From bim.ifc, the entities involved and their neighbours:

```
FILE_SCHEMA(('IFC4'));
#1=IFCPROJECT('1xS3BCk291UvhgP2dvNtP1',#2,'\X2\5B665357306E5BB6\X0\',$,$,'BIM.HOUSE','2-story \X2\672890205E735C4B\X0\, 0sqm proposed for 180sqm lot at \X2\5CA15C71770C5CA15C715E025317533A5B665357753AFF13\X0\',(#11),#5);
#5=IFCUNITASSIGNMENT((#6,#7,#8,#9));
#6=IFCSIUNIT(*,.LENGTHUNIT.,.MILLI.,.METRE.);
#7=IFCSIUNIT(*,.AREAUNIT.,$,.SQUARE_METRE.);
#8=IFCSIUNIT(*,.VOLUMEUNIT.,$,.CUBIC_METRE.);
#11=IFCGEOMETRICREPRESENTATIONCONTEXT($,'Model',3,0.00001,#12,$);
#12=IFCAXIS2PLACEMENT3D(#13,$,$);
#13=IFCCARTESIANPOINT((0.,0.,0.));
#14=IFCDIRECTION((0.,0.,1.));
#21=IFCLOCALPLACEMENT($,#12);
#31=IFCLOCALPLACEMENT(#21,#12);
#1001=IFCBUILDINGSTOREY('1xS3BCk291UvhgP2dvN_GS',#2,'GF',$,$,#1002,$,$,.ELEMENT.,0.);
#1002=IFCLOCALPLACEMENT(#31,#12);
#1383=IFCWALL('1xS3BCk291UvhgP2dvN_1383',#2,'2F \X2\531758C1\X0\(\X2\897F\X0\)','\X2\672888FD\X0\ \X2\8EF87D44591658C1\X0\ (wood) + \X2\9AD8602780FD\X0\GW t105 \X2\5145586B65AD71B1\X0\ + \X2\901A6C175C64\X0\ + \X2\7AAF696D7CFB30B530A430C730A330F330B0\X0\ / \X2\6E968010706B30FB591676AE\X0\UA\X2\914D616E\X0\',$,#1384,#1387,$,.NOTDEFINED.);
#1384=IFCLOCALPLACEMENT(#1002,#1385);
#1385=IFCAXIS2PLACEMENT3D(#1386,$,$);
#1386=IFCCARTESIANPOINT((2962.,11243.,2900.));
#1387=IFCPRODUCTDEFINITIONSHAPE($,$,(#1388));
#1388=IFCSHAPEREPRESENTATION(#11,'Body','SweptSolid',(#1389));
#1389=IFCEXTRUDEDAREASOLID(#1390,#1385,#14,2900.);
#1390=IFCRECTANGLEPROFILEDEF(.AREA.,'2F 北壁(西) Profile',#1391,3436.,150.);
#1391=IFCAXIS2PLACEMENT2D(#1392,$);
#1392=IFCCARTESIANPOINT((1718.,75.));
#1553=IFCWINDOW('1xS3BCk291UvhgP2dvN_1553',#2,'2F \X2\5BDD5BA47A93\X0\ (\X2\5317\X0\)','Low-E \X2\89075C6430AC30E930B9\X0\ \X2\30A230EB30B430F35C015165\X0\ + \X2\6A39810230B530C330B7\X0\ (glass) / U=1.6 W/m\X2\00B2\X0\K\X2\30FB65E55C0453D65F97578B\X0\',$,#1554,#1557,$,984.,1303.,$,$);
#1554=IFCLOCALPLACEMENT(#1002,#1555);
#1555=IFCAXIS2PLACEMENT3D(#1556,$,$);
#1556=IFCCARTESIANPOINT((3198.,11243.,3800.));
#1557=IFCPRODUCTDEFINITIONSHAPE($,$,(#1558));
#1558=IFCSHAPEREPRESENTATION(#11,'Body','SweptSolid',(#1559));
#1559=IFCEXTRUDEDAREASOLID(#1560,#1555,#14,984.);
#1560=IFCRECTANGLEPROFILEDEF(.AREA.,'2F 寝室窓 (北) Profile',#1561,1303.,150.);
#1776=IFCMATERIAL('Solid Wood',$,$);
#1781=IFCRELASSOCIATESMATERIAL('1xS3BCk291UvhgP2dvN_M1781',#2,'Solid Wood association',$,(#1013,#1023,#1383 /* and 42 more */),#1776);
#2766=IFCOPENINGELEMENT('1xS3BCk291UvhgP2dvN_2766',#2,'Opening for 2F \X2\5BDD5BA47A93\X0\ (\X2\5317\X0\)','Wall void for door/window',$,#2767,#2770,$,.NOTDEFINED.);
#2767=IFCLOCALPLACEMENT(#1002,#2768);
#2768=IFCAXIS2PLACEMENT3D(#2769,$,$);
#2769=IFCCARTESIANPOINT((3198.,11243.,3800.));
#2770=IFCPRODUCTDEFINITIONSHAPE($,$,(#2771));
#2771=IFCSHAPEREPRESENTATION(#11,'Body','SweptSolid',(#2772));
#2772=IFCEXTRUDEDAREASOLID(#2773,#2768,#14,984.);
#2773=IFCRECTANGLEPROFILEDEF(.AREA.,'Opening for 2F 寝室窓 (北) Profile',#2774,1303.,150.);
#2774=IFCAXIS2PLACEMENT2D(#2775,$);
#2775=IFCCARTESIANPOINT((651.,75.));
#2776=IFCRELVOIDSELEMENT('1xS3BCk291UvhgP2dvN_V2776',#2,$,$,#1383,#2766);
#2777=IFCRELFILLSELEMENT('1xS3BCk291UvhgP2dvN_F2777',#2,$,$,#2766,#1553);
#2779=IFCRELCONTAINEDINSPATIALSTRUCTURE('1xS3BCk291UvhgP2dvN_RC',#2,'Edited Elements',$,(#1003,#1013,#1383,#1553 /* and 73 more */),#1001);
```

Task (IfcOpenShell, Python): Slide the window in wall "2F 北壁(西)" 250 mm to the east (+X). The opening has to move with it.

```python
import ifcopenshell
import ifcopenshell.api.geometry
import ifcopenshell.util.placement

model = ifcopenshell.open("bim.ifc")

window = model.by_id(1553)
opening = window.FillsVoids[0].RelatingOpeningElement
wall = opening.VoidsElements[0].RelatingBuildingElement

wall_matrix = ifcopenshell.util.placement.get_local_placement(wall.ObjectPlacement)
shift = wall_matrix[:3, 0] * 250.0
before = ifcopenshell.util.placement.get_local_placement(window.ObjectPlacement)[:3, 3].copy()

# The window is not placed relative to its opening, so move both.
for product in (opening, window):
    matrix = ifcopenshell.util.placement.get_local_placement(product.ObjectPlacement)
    matrix[:3, 3] += shift
    ifcopenshell.api.geometry.edit_object_placement(model, product=product, matrix=matrix, is_si=False)

after = ifcopenshell.util.placement.get_local_placement(window.ObjectPlacement)[:3, 3]
print("window moved by", (after - before).round(3) + 0.0)

model.write("bim_rev.ifc")
```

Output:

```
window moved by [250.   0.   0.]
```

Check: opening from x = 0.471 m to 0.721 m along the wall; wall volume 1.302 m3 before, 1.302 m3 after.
